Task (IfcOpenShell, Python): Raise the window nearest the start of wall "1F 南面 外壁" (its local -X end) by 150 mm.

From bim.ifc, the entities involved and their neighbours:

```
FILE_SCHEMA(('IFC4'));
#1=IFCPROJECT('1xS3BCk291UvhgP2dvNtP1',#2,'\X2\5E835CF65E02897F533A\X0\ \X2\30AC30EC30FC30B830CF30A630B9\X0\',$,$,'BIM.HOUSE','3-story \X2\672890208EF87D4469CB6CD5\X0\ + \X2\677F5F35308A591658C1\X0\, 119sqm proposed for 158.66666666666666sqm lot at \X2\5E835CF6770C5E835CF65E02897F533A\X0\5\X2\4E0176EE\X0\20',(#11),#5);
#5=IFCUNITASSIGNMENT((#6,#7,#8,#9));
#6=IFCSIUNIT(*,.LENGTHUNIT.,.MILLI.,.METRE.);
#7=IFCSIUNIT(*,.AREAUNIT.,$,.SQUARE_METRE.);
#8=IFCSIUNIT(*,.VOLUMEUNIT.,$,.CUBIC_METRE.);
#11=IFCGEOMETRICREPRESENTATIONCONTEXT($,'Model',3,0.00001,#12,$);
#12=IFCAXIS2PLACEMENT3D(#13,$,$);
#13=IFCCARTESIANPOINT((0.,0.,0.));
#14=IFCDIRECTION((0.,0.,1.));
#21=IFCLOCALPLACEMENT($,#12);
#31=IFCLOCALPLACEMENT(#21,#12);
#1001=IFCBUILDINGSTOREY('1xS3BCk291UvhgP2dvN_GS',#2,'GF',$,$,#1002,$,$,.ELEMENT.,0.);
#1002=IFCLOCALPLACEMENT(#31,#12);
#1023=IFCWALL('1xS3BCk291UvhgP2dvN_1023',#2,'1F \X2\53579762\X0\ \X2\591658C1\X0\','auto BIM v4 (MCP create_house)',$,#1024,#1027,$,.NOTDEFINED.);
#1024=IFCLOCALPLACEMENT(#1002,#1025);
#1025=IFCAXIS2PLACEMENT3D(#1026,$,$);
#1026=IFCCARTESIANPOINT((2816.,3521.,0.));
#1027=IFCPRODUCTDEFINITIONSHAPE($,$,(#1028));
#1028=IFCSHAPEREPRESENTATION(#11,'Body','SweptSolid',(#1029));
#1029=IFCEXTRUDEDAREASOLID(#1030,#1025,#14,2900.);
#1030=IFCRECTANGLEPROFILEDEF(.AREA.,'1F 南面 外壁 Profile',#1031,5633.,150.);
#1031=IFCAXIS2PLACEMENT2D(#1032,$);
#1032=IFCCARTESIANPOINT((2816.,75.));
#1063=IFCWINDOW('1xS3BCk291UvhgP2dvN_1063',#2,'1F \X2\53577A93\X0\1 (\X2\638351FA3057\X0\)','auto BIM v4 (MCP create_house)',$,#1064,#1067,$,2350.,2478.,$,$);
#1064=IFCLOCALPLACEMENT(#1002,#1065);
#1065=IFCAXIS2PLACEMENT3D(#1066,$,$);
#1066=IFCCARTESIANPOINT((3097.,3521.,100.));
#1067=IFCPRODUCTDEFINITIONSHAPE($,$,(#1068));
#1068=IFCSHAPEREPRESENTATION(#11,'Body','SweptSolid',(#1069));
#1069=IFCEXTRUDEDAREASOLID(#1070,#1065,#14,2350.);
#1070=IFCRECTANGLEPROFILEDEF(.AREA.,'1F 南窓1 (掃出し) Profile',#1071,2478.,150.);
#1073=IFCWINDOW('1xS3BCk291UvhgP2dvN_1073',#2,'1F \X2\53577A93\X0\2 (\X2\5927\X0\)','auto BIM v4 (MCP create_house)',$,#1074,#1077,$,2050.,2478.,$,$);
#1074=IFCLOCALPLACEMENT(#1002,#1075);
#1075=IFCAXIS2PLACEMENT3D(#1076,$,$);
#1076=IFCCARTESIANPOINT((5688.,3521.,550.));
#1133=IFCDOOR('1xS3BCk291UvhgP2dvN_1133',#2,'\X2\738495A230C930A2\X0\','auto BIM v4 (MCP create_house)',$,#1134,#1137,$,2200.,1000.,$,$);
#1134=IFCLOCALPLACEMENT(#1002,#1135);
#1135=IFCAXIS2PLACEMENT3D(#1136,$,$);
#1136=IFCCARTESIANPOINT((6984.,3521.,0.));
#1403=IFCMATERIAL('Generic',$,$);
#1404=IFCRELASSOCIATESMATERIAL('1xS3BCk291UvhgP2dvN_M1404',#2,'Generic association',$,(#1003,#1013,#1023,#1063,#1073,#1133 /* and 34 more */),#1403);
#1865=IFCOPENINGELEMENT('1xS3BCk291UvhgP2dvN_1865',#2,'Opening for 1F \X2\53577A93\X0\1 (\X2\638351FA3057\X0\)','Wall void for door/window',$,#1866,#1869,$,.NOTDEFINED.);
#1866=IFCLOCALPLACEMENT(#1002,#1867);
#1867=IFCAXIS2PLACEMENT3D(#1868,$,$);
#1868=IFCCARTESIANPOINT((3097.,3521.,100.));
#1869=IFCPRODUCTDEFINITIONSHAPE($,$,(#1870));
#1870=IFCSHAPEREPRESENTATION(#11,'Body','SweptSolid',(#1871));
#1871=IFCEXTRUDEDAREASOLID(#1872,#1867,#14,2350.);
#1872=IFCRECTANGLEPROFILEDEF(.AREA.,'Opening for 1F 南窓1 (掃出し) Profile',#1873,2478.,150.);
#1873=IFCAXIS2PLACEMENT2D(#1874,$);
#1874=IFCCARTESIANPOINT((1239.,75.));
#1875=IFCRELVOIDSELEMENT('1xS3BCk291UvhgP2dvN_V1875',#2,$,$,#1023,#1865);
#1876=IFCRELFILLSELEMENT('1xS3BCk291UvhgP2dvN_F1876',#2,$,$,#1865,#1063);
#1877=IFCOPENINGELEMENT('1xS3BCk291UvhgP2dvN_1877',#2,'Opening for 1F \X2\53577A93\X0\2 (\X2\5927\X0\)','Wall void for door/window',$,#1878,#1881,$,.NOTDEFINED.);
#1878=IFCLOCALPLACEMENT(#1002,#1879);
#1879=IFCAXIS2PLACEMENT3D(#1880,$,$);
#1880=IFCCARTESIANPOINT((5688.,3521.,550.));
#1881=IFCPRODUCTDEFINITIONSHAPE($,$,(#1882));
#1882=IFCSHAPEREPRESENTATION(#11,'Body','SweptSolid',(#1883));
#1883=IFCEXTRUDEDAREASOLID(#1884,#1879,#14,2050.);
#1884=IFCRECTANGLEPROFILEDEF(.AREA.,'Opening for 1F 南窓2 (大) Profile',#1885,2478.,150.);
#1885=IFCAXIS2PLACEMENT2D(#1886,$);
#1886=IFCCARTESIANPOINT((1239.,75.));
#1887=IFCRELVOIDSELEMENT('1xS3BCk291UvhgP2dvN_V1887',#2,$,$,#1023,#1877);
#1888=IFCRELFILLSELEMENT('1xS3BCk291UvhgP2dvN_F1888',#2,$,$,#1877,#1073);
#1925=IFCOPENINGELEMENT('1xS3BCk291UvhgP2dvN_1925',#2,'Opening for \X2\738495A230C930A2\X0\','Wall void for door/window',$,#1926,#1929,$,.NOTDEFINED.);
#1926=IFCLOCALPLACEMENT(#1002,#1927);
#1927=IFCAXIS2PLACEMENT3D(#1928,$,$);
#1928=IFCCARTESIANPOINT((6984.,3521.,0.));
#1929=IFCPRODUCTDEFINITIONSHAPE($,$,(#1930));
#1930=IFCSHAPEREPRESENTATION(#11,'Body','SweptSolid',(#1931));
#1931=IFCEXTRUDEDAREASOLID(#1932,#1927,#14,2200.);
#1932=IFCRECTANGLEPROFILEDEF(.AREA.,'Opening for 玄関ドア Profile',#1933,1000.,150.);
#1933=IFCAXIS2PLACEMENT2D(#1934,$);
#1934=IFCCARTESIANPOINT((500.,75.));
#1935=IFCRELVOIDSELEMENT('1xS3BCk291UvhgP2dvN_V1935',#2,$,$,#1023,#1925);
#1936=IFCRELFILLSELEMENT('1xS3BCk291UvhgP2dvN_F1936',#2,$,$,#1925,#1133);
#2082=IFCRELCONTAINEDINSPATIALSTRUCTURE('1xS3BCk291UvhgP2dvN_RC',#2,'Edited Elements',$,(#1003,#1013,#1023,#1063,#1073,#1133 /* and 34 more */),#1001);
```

```python
import numpy as np
import ifcopenshell
import ifcopenshell.api.geometry
import ifcopenshell.util.placement
import ifcopenshell.util.unit

model = ifcopenshell.open("bim.ifc")
unit_scale = ifcopenshell.util.unit.calculate_unit_scale(model)

window = model.by_guid("1xS3BCk291UvhgP2dvN_1063")
opening = window.FillsVoids[0].RelatingOpeningElement
dz = 0.15 / unit_scale

shift = np.array([0.0, 0.0, dz])
# The window is not placed relative to its opening, so move both.
for product in (opening, window):
    matrix = ifcopenshell.util.placement.get_local_placement(product.ObjectPlacement)
    matrix[:3, 3] += shift
    ifcopenshell.api.geometry.edit_object_placement(model, product=product, matrix=matrix, is_si=False)

print(f"moved by {dz * unit_scale:+.3f} m")

model.write("bim-out.ifc")
```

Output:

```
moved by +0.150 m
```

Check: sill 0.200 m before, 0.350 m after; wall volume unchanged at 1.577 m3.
